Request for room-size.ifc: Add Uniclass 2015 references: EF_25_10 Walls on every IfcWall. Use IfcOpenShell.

First a look at what the model holds.

```python
import ifcopenshell

model = ifcopenshell.open("room-size.ifc")
print(model.schema)
print("classifications:", [c.Name for c in model.by_type("IfcClassification")])
for ifc_class in ("IfcDoor", "IfcRoof", "IfcStair", "IfcWall", "IfcWindow"):
    print(ifc_class, len(model.by_type(ifc_class)))
```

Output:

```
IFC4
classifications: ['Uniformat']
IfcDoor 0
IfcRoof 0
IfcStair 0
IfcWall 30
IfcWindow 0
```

```python
import ifcopenshell
import ifcopenshell.api.classification

model = ifcopenshell.open("room-size.ifc")

system = ifcopenshell.api.classification.add_classification(model, classification="Uniclass 2015")

codes = {
    "IfcWall": ("EF_25_10", "Walls"),
}
for ifc_class, (code, name) in codes.items():
    products = model.by_type(ifc_class)
    ifcopenshell.api.classification.add_reference(
        model, products=products, classification=system, identification=code, name=name
    )
    print(code, len(products))

model.write("room-size_edited.ifc")
```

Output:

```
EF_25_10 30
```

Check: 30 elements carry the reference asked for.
